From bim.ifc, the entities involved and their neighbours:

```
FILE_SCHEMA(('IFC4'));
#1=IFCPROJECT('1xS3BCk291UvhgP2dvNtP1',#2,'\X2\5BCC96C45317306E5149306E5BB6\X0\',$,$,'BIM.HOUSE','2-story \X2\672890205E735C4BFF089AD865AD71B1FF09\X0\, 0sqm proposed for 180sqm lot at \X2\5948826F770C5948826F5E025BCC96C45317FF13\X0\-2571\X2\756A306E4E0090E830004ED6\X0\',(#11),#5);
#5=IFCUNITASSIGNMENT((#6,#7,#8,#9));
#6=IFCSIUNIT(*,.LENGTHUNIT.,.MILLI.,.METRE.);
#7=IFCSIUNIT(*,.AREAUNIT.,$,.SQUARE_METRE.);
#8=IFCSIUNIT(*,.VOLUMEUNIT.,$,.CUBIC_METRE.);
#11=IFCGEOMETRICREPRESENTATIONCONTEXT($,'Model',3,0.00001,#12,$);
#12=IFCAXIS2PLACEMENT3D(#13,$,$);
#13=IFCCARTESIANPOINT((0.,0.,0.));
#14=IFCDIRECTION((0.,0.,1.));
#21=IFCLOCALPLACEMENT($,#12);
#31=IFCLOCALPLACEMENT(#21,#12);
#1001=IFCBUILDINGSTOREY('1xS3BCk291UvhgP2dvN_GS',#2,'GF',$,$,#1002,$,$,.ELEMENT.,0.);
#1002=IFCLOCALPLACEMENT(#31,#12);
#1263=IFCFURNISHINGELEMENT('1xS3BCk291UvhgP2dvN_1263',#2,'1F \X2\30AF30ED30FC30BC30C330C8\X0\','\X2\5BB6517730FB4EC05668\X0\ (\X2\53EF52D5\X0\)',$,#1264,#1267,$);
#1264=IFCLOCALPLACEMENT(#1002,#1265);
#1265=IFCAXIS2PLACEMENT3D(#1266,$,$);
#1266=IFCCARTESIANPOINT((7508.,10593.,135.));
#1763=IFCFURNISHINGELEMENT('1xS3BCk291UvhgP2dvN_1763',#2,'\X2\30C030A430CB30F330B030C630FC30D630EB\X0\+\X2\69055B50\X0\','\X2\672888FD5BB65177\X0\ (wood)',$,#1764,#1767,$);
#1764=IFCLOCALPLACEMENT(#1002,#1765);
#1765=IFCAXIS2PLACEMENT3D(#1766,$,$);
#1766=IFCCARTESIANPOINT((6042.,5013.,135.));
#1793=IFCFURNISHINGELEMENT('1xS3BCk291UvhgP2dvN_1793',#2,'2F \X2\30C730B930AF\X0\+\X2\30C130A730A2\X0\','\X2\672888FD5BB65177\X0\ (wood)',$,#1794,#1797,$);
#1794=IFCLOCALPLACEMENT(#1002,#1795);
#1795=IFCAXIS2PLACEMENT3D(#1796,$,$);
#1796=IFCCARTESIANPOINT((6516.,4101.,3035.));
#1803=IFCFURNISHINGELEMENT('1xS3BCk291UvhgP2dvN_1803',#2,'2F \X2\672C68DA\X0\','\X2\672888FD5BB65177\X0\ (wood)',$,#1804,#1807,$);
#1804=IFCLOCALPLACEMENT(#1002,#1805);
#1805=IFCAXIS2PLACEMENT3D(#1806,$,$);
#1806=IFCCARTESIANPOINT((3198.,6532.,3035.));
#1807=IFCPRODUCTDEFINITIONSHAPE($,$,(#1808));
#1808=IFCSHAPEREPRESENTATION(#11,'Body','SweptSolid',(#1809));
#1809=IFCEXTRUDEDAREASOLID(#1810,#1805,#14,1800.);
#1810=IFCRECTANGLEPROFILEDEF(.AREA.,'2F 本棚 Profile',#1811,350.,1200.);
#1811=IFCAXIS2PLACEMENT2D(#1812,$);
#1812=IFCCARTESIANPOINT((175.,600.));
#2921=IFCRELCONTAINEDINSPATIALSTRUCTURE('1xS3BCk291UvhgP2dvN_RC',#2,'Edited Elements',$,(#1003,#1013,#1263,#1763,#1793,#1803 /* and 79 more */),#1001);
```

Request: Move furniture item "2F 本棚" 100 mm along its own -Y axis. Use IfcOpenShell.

```python
import ifcopenshell
import ifcopenshell.api.geometry
import ifcopenshell.util.placement
import ifcopenshell.util.unit

model = ifcopenshell.open("bim.ifc")
unit_scale = ifcopenshell.util.unit.calculate_unit_scale(model)

item = model.by_id(1803)
matrix = ifcopenshell.util.placement.get_local_placement(item.ObjectPlacement)
matrix[:3, 3] -= matrix[:3, 1] * 0.1 / unit_scale
ifcopenshell.api.geometry.edit_object_placement(model, product=item, matrix=matrix, is_si=False)

print(ifcopenshell.util.placement.get_local_placement(item.ObjectPlacement).round(3) + 0.0)

model.write("bim_rev.ifc")
```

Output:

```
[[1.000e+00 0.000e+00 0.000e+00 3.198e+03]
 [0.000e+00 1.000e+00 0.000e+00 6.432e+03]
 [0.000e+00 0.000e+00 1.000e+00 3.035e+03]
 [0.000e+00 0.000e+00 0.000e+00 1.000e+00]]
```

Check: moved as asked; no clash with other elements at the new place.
